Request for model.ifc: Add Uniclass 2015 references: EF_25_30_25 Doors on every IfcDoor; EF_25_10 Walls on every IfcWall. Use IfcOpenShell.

First a look at what the model holds.

```python
import ifcopenshell

model = ifcopenshell.open("model.ifc")
print(model.schema)
print("classifications:", [c.Name for c in model.by_type("IfcClassification")])
for ifc_class in ("IfcDoor", "IfcRoof", "IfcStair", "IfcWall", "IfcWindow"):
    print(ifc_class, len(model.by_type(ifc_class)))
```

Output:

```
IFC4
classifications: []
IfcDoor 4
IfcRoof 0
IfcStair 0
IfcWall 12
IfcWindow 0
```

```python
import ifcopenshell
import ifcopenshell.api.classification

model = ifcopenshell.open("model.ifc")

system = ifcopenshell.api.classification.add_classification(model, classification="Uniclass 2015")

codes = {
    "IfcDoor": ("EF_25_30_25", "Doors"),
    "IfcWall": ("EF_25_10", "Walls"),
}
for ifc_class, (code, name) in codes.items():
    products = model.by_type(ifc_class)
    ifcopenshell.api.classification.add_reference(
        model, products=products, classification=system, identification=code, name=name
    )
    print(code, len(products))

model.write("model-out.ifc")
```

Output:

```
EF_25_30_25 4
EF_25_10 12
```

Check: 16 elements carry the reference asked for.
